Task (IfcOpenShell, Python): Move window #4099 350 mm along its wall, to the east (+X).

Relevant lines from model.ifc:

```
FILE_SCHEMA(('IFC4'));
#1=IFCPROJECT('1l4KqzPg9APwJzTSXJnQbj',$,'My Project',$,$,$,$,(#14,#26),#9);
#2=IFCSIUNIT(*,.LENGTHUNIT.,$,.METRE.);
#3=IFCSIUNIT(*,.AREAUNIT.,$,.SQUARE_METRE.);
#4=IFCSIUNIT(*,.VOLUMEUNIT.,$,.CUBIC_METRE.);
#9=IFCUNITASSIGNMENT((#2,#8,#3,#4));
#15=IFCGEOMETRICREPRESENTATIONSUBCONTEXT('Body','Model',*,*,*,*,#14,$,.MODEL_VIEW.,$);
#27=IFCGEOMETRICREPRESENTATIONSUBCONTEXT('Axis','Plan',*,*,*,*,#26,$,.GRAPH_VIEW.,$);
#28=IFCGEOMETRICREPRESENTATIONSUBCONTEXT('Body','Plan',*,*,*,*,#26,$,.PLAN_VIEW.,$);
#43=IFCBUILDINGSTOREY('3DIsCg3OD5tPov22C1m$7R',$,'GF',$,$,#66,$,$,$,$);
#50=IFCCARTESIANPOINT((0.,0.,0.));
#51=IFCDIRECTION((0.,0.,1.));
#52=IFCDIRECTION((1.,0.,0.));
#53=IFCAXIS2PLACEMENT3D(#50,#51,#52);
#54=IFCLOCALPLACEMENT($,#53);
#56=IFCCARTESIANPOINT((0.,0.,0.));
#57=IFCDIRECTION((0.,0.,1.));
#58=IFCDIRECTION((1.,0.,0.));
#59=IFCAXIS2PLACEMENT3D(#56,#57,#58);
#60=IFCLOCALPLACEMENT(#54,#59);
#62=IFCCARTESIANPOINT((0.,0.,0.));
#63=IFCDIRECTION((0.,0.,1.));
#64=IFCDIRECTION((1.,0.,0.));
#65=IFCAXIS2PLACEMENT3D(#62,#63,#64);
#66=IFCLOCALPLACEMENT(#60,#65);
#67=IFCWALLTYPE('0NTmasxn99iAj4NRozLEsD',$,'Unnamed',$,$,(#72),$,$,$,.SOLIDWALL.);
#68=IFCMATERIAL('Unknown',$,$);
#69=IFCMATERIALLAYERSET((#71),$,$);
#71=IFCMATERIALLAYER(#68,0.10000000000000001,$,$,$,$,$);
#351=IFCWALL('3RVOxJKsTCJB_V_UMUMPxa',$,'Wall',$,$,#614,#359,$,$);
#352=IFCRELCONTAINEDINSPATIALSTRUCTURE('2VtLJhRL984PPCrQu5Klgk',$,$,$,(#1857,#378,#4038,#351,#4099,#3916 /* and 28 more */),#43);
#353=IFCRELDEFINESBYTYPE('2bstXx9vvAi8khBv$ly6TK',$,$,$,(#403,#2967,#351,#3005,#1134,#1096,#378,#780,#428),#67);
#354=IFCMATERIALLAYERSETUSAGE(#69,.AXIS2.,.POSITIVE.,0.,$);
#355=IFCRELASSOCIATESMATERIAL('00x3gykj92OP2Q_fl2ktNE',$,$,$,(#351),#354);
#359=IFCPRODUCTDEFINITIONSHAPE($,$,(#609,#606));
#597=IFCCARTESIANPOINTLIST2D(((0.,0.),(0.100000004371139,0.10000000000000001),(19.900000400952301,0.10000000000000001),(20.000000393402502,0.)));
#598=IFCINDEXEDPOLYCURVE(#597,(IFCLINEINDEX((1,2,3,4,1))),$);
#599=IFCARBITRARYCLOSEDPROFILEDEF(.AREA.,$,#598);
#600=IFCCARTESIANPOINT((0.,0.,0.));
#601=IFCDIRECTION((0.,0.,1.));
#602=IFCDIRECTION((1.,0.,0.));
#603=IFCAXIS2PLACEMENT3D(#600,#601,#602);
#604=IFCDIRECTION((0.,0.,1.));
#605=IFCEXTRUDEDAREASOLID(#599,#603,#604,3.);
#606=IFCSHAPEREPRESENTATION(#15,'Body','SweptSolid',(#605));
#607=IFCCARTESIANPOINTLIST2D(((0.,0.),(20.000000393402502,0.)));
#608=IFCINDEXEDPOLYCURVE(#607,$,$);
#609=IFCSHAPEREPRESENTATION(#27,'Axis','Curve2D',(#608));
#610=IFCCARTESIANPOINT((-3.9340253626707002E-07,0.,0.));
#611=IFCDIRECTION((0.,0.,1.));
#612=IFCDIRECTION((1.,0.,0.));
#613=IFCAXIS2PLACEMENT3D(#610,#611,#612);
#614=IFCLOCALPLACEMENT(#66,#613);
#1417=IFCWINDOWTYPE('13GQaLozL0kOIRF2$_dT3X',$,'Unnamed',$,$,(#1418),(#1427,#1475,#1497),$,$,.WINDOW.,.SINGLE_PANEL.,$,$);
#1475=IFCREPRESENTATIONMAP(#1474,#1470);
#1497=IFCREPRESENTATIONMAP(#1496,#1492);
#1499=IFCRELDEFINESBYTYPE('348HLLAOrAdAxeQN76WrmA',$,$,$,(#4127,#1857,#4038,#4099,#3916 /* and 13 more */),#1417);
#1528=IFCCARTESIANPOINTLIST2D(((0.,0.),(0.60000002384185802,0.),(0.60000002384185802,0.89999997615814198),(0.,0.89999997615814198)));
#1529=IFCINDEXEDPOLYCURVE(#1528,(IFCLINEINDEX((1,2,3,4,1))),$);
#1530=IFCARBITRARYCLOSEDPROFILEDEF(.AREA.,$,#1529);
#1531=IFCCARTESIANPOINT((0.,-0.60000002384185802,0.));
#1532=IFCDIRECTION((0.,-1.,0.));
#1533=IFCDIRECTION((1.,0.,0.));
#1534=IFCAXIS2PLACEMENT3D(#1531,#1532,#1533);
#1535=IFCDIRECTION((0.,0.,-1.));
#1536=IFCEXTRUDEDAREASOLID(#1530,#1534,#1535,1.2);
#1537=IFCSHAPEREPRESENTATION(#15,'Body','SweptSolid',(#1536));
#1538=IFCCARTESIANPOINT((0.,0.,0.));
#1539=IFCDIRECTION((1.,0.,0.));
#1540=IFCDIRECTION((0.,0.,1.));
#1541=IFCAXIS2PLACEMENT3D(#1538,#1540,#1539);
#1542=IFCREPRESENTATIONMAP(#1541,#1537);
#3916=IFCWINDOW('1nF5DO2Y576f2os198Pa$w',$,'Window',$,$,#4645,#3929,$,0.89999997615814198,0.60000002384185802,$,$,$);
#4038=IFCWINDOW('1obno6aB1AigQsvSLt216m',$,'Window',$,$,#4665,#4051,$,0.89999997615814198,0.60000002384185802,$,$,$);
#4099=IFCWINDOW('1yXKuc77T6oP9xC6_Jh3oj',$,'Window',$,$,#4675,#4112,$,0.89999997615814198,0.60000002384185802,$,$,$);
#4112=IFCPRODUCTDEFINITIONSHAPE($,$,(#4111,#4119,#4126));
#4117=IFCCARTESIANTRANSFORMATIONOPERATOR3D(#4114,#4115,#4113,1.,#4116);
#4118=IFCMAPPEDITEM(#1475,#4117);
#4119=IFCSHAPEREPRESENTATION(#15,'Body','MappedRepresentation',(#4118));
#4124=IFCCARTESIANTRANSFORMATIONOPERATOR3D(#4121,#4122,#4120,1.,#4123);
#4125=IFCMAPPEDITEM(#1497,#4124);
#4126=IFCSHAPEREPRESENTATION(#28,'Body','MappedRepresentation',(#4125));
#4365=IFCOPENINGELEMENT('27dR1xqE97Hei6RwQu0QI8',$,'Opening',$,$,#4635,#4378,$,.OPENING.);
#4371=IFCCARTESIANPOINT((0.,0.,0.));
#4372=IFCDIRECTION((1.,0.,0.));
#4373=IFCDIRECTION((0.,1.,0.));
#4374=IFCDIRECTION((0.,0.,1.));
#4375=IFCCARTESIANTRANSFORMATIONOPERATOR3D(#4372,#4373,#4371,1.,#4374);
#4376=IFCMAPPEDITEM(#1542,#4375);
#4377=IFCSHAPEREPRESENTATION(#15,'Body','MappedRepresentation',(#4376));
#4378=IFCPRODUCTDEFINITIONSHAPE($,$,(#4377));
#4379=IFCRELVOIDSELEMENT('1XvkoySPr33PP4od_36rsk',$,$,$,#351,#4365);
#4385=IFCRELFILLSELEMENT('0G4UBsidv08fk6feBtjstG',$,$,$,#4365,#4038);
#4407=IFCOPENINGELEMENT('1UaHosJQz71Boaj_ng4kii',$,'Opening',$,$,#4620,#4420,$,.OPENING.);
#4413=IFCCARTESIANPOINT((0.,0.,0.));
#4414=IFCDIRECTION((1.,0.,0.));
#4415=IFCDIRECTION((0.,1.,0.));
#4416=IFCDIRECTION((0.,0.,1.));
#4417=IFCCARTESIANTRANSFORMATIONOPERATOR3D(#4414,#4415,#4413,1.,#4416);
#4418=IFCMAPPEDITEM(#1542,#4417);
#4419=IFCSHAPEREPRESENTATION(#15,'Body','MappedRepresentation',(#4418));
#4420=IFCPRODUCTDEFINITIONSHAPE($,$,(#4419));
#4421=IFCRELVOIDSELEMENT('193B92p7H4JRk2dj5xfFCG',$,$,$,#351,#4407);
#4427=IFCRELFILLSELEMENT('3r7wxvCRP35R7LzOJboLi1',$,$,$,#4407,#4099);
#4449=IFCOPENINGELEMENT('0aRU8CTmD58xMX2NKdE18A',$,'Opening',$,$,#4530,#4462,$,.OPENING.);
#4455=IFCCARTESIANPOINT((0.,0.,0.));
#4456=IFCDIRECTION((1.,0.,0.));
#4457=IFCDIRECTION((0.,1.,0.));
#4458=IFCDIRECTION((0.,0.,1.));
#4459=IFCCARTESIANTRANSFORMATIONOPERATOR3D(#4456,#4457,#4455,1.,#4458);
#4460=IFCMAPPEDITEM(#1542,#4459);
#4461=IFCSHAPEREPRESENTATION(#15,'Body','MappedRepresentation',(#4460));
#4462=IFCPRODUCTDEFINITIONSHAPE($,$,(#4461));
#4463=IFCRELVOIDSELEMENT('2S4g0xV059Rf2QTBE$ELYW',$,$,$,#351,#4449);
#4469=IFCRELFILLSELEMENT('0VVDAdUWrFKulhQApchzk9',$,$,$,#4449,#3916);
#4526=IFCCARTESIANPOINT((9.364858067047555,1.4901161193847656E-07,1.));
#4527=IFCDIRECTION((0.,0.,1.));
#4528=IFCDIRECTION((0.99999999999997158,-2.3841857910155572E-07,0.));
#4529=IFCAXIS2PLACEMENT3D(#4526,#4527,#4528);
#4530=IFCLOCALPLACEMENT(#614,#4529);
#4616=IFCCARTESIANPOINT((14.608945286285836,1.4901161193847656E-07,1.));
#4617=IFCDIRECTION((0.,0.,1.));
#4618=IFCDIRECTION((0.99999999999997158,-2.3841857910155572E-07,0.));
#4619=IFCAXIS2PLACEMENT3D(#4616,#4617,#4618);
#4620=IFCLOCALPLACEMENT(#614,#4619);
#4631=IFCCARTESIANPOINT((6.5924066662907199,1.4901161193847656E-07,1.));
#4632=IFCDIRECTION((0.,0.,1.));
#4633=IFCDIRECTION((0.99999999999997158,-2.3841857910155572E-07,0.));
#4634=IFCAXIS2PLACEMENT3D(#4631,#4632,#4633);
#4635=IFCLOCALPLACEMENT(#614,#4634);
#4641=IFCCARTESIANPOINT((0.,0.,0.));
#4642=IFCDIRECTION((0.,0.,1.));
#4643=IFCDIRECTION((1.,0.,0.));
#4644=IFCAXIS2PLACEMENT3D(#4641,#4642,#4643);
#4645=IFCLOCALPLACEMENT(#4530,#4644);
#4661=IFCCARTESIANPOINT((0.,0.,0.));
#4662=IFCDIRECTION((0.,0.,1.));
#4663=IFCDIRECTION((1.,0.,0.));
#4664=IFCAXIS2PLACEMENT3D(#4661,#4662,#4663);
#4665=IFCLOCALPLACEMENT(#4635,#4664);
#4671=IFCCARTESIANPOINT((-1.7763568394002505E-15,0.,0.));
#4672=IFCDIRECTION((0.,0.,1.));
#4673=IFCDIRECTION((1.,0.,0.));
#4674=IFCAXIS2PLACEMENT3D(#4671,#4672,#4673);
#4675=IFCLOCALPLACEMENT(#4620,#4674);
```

```python
import ifcopenshell
import ifcopenshell.api.geometry
import ifcopenshell.util.placement
import ifcopenshell.util.unit

model = ifcopenshell.open("model.ifc")
unit_scale = ifcopenshell.util.unit.calculate_unit_scale(model)

window = model.by_guid("1yXKuc77T6oP9xC6_Jh3oj")
opening = window.FillsVoids[0].RelatingOpeningElement
wall = opening.VoidsElements[0].RelatingBuildingElement

wall_matrix = ifcopenshell.util.placement.get_local_placement(wall.ObjectPlacement)
shift = wall_matrix[:3, 0] * 0.35 / unit_scale
before = ifcopenshell.util.placement.get_local_placement(window.ObjectPlacement)[:3, 3].copy()

# The window is placed relative to its opening, so it follows when the opening moves.
matrix = ifcopenshell.util.placement.get_local_placement(opening.ObjectPlacement)
matrix[:3, 3] += shift
ifcopenshell.api.geometry.edit_object_placement(
    model, product=opening, matrix=matrix, is_si=False, should_transform_children=True
)

after = ifcopenshell.util.placement.get_local_placement(window.ObjectPlacement)[:3, 3]
print("window moved by", (after - before).round(3) + 0.0)

model.write("model_updated.ifc")
```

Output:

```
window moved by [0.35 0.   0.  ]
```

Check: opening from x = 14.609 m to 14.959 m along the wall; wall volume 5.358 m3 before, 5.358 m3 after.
